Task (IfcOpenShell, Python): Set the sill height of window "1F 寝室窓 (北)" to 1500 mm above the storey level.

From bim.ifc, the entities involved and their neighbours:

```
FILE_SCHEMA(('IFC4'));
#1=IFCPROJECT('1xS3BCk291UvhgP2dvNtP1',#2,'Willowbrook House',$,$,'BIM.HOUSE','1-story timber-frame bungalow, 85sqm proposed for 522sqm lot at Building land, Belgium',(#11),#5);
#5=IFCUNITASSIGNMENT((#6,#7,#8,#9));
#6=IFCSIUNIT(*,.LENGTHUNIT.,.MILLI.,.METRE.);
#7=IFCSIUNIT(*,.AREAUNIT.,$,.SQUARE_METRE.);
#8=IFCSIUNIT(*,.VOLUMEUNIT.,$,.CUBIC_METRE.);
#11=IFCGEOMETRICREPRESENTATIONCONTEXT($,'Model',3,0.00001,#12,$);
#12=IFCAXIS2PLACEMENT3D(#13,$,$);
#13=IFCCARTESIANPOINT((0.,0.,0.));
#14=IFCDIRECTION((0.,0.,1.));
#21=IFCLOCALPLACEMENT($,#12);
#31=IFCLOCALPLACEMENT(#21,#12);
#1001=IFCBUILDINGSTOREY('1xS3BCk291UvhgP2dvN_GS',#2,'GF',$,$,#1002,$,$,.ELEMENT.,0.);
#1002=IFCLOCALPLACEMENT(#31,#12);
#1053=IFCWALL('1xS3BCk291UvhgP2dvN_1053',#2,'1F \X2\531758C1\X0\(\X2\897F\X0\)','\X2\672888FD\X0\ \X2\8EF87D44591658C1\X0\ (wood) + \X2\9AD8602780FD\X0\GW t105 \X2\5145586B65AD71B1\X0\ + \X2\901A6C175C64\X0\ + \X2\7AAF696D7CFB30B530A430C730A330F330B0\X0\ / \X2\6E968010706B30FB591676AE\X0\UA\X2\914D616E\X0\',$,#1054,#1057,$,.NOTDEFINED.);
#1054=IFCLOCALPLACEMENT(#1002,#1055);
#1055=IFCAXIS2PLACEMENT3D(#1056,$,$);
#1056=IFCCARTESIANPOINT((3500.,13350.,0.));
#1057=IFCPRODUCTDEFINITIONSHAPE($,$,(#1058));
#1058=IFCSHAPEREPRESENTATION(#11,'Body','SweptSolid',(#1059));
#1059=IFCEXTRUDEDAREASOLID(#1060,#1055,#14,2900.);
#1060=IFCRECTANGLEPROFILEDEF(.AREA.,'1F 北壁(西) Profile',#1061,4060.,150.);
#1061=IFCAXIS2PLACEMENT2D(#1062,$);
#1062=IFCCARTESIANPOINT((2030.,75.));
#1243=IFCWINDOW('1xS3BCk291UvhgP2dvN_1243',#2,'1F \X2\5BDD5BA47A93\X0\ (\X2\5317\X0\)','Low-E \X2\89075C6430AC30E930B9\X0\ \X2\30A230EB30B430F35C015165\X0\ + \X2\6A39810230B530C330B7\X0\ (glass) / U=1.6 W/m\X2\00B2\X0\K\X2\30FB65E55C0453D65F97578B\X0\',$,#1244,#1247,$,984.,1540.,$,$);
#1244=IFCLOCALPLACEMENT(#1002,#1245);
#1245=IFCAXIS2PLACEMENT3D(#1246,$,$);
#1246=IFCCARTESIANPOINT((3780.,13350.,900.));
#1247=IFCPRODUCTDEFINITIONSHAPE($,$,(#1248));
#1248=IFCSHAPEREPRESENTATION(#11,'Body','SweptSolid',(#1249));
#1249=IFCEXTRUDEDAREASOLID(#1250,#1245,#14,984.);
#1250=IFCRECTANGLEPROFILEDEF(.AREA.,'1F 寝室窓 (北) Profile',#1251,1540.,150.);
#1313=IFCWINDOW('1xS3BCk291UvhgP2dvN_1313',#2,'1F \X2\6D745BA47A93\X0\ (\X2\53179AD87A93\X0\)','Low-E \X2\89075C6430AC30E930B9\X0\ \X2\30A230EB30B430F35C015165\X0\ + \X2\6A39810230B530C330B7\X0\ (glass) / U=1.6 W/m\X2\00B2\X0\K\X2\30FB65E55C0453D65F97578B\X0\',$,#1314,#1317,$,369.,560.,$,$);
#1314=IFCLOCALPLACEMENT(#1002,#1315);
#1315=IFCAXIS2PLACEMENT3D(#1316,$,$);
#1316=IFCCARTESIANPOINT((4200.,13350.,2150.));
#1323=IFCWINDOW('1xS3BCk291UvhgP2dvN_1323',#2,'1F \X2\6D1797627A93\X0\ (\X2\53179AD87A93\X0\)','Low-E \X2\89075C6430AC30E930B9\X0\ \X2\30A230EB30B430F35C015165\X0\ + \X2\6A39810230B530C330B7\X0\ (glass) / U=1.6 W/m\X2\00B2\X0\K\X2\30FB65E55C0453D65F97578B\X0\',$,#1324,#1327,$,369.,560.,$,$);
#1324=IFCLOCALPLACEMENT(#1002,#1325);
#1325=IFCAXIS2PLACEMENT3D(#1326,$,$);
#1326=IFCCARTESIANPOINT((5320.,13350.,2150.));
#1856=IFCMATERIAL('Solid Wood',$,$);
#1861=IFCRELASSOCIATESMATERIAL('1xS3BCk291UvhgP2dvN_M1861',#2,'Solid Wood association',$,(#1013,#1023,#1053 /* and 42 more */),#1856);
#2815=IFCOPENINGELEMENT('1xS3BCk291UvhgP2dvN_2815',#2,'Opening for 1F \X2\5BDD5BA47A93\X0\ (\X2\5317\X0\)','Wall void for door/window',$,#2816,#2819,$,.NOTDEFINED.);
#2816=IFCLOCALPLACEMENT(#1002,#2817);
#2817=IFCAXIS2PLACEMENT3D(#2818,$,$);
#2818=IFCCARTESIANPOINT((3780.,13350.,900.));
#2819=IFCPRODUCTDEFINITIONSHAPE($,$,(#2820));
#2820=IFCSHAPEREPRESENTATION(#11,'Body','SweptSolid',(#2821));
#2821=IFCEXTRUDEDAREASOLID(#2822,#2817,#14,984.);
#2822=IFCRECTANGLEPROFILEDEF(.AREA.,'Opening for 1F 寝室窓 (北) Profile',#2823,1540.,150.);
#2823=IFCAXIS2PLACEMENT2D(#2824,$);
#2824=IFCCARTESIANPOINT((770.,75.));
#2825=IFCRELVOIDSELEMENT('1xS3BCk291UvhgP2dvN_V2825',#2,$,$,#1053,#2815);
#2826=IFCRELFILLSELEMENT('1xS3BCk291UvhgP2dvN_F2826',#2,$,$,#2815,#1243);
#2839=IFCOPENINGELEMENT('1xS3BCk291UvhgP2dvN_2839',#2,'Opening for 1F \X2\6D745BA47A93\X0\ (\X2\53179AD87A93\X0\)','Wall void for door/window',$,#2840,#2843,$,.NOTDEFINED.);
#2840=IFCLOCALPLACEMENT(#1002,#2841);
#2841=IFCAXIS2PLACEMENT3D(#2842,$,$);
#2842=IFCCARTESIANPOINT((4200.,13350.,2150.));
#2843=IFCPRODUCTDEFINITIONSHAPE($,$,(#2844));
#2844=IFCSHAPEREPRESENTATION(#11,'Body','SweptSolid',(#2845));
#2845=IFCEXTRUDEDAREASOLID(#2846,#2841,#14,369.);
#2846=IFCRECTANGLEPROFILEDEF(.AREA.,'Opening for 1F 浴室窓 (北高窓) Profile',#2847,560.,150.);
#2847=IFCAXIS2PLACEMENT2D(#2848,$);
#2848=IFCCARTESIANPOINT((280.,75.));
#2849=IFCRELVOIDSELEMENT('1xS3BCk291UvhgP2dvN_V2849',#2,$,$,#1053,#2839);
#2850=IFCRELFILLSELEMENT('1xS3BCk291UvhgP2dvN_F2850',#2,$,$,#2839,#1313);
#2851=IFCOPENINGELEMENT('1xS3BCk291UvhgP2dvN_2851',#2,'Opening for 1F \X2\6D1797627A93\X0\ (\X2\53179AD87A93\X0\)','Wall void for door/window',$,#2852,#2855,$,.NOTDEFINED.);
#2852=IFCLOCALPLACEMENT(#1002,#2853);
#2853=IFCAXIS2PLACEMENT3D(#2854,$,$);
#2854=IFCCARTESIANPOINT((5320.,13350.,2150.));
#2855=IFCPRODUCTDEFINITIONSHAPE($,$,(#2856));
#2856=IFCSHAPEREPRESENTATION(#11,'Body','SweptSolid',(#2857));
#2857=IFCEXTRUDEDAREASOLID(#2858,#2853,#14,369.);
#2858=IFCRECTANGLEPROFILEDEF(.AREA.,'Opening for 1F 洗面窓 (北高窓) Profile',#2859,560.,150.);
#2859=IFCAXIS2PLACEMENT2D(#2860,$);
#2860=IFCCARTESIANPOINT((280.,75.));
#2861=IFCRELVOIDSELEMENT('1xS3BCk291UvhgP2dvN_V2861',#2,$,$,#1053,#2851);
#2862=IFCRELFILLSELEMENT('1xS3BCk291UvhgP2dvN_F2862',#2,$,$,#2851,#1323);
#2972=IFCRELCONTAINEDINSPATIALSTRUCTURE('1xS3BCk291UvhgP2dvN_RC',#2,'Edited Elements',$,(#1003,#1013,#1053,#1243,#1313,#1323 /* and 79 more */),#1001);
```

```python
import numpy as np
import ifcopenshell
import ifcopenshell.api.geometry
import ifcopenshell.geom
import ifcopenshell.util.element
import ifcopenshell.util.placement
import ifcopenshell.util.shape
import ifcopenshell.util.unit

model = ifcopenshell.open("bim.ifc")
unit_scale = ifcopenshell.util.unit.calculate_unit_scale(model)

window = model.by_guid("1xS3BCk291UvhgP2dvN_1243")
opening = window.FillsVoids[0].RelatingOpeningElement
storey = ifcopenshell.util.element.get_container(window, ifc_class="IfcBuildingStorey")
level = ifcopenshell.util.placement.get_local_placement(storey.ObjectPlacement)[2, 3]

# The opening's origin need not be at the sill, so measure its lowest point.
shape = ifcopenshell.geom.create_shape(ifcopenshell.geom.settings(), opening)
bottom = ifcopenshell.util.shape.get_shape_bottom_elevation(shape, shape.geometry) / unit_scale
dz = level + 1500.0 - bottom

shift = np.array([0.0, 0.0, dz])
# The window is not placed relative to its opening, so move both.
for product in (opening, window):
    matrix = ifcopenshell.util.placement.get_local_placement(product.ObjectPlacement)
    matrix[:3, 3] += shift
    ifcopenshell.api.geometry.edit_object_placement(model, product=product, matrix=matrix, is_si=False)

print(f"moved by {dz * unit_scale:+.3f} m")

model.write("bim_edited.ifc")
```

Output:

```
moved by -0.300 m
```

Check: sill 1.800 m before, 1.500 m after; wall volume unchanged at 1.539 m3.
